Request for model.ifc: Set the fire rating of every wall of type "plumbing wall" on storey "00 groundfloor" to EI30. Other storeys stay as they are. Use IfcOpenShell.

First a look at what the model holds.

```python
import ifcopenshell
import ifcopenshell.util.element

model = ifcopenshell.open("model.ifc")
print(model.schema)
storey = next(s for s in model.by_type("IfcBuildingStorey") if s.Name == "00 groundfloor")
walls = [e for e in ifcopenshell.util.element.get_decomposition(storey) if e.is_a("IfcWall")]
seen = {}
for e in walls:
    element_type = ifcopenshell.util.element.get_type(e)
    key = (element_type.Name if element_type != e and element_type else None, ifcopenshell.util.element.get_pset(e, "Pset_WallCommon", "FireRating"))
    seen[key] = seen.get(key, 0) + 1
for (name, value), count in sorted(seen.items(), key=str):
    print(count, "x", name, "|", value)
```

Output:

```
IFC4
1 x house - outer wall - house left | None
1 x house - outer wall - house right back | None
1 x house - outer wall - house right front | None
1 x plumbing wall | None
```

```python
import ifcopenshell
import ifcopenshell.api.pset
import ifcopenshell.util.element

model = ifcopenshell.open("model.ifc")

storey = next(s for s in model.by_type("IfcBuildingStorey") if s.Name == "00 groundfloor")
walls = [e for e in ifcopenshell.util.element.get_decomposition(storey) if e.is_a("IfcWall")]

count = 0
for e in walls:
    element_type = ifcopenshell.util.element.get_type(e)
    if element_type in (None, e) or element_type.Name != "plumbing wall":
        continue
    # add_pset returns the element's existing set when there is one.
    pset = ifcopenshell.api.pset.add_pset(model, product=e, name="Pset_WallCommon")
    ifcopenshell.api.pset.edit_pset(model, pset=pset, properties={"FireRating": "EI30"})
    count += 1

print(count, "walls updated")

model.write("model_rev.ifc")
```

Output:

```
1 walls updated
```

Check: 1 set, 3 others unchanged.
